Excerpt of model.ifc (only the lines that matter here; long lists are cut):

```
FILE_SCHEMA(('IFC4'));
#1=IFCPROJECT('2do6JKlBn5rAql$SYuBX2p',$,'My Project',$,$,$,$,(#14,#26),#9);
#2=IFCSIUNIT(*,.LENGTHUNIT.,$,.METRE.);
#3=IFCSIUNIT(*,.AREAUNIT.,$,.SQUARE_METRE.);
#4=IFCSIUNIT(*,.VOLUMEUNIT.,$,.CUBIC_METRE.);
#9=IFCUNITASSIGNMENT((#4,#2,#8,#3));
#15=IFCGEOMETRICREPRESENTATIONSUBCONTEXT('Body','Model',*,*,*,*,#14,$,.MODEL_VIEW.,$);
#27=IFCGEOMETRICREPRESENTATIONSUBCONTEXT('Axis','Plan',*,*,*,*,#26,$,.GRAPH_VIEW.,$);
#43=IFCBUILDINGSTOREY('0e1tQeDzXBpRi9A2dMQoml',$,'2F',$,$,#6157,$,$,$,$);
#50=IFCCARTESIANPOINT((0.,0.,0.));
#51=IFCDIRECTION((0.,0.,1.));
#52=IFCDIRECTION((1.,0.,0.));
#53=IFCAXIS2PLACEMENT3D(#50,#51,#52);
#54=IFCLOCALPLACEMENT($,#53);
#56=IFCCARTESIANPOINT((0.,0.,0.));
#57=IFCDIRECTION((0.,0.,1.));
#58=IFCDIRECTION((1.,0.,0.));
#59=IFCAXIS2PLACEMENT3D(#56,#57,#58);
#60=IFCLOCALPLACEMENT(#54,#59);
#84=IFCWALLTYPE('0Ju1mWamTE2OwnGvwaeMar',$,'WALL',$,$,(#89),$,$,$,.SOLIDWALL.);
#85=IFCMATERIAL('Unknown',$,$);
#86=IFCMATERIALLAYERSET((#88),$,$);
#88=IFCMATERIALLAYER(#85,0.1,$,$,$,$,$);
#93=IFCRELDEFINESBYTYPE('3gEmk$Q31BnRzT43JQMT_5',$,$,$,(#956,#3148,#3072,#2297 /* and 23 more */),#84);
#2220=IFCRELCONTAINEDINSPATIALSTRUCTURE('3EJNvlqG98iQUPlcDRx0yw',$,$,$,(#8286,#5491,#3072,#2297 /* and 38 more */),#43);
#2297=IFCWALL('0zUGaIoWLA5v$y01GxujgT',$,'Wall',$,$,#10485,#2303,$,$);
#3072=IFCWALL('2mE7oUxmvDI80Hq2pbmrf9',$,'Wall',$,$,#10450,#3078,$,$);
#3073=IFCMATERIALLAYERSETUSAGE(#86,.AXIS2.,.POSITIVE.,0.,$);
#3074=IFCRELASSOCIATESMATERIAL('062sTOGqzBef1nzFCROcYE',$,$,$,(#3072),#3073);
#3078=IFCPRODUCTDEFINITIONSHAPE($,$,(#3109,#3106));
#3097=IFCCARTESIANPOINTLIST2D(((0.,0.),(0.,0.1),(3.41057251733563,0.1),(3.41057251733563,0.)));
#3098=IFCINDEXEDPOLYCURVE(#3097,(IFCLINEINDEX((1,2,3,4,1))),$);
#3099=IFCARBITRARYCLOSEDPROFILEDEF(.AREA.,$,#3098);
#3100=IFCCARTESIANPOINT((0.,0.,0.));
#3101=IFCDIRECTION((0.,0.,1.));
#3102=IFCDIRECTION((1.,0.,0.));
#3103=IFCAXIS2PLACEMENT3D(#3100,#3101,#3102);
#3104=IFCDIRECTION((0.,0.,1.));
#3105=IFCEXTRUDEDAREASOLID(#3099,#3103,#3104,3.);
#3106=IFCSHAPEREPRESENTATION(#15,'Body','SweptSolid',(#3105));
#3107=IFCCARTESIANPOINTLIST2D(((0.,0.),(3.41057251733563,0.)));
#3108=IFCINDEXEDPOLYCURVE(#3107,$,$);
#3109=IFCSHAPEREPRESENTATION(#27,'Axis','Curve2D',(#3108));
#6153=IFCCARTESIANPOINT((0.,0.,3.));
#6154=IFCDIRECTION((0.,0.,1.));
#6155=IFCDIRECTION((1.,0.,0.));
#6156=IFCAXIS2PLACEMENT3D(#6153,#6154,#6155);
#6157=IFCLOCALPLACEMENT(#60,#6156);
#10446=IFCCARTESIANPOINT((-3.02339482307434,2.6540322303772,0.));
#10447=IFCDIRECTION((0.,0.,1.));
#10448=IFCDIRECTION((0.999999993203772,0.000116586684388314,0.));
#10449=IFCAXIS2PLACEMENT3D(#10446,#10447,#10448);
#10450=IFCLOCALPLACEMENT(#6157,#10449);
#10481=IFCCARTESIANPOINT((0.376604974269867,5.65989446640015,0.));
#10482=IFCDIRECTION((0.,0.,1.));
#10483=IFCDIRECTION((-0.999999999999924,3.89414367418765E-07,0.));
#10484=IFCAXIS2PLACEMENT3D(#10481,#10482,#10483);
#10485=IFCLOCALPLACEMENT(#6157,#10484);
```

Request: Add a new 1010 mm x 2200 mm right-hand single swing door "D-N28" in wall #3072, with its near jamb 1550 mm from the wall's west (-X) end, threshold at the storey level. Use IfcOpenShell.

```python
import numpy as np
import ifcopenshell
import ifcopenshell.api.feature
import ifcopenshell.api.geometry
import ifcopenshell.api.root
import ifcopenshell.api.spatial
import ifcopenshell.geom
import ifcopenshell.util.element
import ifcopenshell.util.placement
import ifcopenshell.util.representation
import ifcopenshell.util.shape
import ifcopenshell.util.unit

model = ifcopenshell.open("model.ifc")
unit_scale = ifcopenshell.util.unit.calculate_unit_scale(model)
settings = ifcopenshell.geom.settings()


def volume(element):
    """Net volume in cubic metres, openings subtracted."""
    shape = ifcopenshell.geom.create_shape(settings, element)
    return ifcopenshell.util.shape.get_volume(shape.geometry)


wall = model.by_guid("2mE7oUxmvDI80Hq2pbmrf9")
storey = ifcopenshell.util.element.get_container(wall, ifc_class="IfcBuildingStorey")
context = ifcopenshell.util.representation.get_context(model, "Model", "Body", "MODEL_VIEW")
before = volume(wall)

width, height, from_end, sill = 1.01, 2.2, 1.55, 0.0  # metres

# The wall runs along its own X axis, and the end named is its -X end.
wall_shape = ifcopenshell.geom.create_shape(settings, wall)
x, y, z = ifcopenshell.util.shape.get_vertices(wall_shape.geometry).T
start = x.min() + from_end
face, thickness = float(y.min()), float(y.max() - y.min())
wall_matrix = ifcopenshell.util.placement.get_local_placement(wall.ObjectPlacement)
level = ifcopenshell.util.placement.get_local_placement(storey.ObjectPlacement)[2, 3]


def in_wall(x, y):
    """Placement at x, y metres in the wall's axes, at sill height."""
    matrix = wall_matrix.copy()
    matrix[:, 3] = wall_matrix @ np.array([x / unit_scale, y / unit_scale, 0.0, 1.0])
    matrix[2, 3] = level + sill / unit_scale
    return matrix


# Opening: a box that overshoots both wall faces by 50 mm.
opening = ifcopenshell.api.root.create_entity(model, ifc_class="IfcOpeningElement", predefined_type="OPENING")
box = ifcopenshell.api.geometry.add_wall_representation(
    model, context=context, length=width, height=height, thickness=thickness + 0.1
)
ifcopenshell.api.geometry.assign_representation(model, product=opening, representation=box)
ifcopenshell.api.geometry.edit_object_placement(model, product=opening, matrix=in_wall(start, face - 0.05), is_si=False)
ifcopenshell.api.feature.add_feature(model, feature=opening, element=wall)

door = ifcopenshell.api.root.create_entity(model, ifc_class="IfcDoor", name="D-N28", predefined_type="DOOR")
door.OverallWidth, door.OverallHeight = width / unit_scale, height / unit_scale
door.OperationType = "SINGLE_SWING_RIGHT"
body = ifcopenshell.api.geometry.add_door_representation(
    model,
    context=context,
    overall_width=door.OverallWidth,
    overall_height=door.OverallHeight,
    operation_type="SINGLE_SWING_RIGHT",
    lining_properties={"LiningDepth": thickness / unit_scale, "ThresholdDepth": thickness / unit_scale},
)
ifcopenshell.api.geometry.assign_representation(model, product=door, representation=body)
ifcopenshell.api.spatial.assign_container(model, products=[door], relating_structure=storey)
ifcopenshell.api.feature.add_filling(model, opening=opening, element=door)

# The lining spans the wall, so the door starts at the wall face.
ifcopenshell.api.geometry.edit_object_placement(model, product=door, matrix=in_wall(start, face), is_si=False)

after = volume(wall)

print(f"wall volume {before:.3f} -> {after:.3f} m3")

model.write("model_edited.ifc")
```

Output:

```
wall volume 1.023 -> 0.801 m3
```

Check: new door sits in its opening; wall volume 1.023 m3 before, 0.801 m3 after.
